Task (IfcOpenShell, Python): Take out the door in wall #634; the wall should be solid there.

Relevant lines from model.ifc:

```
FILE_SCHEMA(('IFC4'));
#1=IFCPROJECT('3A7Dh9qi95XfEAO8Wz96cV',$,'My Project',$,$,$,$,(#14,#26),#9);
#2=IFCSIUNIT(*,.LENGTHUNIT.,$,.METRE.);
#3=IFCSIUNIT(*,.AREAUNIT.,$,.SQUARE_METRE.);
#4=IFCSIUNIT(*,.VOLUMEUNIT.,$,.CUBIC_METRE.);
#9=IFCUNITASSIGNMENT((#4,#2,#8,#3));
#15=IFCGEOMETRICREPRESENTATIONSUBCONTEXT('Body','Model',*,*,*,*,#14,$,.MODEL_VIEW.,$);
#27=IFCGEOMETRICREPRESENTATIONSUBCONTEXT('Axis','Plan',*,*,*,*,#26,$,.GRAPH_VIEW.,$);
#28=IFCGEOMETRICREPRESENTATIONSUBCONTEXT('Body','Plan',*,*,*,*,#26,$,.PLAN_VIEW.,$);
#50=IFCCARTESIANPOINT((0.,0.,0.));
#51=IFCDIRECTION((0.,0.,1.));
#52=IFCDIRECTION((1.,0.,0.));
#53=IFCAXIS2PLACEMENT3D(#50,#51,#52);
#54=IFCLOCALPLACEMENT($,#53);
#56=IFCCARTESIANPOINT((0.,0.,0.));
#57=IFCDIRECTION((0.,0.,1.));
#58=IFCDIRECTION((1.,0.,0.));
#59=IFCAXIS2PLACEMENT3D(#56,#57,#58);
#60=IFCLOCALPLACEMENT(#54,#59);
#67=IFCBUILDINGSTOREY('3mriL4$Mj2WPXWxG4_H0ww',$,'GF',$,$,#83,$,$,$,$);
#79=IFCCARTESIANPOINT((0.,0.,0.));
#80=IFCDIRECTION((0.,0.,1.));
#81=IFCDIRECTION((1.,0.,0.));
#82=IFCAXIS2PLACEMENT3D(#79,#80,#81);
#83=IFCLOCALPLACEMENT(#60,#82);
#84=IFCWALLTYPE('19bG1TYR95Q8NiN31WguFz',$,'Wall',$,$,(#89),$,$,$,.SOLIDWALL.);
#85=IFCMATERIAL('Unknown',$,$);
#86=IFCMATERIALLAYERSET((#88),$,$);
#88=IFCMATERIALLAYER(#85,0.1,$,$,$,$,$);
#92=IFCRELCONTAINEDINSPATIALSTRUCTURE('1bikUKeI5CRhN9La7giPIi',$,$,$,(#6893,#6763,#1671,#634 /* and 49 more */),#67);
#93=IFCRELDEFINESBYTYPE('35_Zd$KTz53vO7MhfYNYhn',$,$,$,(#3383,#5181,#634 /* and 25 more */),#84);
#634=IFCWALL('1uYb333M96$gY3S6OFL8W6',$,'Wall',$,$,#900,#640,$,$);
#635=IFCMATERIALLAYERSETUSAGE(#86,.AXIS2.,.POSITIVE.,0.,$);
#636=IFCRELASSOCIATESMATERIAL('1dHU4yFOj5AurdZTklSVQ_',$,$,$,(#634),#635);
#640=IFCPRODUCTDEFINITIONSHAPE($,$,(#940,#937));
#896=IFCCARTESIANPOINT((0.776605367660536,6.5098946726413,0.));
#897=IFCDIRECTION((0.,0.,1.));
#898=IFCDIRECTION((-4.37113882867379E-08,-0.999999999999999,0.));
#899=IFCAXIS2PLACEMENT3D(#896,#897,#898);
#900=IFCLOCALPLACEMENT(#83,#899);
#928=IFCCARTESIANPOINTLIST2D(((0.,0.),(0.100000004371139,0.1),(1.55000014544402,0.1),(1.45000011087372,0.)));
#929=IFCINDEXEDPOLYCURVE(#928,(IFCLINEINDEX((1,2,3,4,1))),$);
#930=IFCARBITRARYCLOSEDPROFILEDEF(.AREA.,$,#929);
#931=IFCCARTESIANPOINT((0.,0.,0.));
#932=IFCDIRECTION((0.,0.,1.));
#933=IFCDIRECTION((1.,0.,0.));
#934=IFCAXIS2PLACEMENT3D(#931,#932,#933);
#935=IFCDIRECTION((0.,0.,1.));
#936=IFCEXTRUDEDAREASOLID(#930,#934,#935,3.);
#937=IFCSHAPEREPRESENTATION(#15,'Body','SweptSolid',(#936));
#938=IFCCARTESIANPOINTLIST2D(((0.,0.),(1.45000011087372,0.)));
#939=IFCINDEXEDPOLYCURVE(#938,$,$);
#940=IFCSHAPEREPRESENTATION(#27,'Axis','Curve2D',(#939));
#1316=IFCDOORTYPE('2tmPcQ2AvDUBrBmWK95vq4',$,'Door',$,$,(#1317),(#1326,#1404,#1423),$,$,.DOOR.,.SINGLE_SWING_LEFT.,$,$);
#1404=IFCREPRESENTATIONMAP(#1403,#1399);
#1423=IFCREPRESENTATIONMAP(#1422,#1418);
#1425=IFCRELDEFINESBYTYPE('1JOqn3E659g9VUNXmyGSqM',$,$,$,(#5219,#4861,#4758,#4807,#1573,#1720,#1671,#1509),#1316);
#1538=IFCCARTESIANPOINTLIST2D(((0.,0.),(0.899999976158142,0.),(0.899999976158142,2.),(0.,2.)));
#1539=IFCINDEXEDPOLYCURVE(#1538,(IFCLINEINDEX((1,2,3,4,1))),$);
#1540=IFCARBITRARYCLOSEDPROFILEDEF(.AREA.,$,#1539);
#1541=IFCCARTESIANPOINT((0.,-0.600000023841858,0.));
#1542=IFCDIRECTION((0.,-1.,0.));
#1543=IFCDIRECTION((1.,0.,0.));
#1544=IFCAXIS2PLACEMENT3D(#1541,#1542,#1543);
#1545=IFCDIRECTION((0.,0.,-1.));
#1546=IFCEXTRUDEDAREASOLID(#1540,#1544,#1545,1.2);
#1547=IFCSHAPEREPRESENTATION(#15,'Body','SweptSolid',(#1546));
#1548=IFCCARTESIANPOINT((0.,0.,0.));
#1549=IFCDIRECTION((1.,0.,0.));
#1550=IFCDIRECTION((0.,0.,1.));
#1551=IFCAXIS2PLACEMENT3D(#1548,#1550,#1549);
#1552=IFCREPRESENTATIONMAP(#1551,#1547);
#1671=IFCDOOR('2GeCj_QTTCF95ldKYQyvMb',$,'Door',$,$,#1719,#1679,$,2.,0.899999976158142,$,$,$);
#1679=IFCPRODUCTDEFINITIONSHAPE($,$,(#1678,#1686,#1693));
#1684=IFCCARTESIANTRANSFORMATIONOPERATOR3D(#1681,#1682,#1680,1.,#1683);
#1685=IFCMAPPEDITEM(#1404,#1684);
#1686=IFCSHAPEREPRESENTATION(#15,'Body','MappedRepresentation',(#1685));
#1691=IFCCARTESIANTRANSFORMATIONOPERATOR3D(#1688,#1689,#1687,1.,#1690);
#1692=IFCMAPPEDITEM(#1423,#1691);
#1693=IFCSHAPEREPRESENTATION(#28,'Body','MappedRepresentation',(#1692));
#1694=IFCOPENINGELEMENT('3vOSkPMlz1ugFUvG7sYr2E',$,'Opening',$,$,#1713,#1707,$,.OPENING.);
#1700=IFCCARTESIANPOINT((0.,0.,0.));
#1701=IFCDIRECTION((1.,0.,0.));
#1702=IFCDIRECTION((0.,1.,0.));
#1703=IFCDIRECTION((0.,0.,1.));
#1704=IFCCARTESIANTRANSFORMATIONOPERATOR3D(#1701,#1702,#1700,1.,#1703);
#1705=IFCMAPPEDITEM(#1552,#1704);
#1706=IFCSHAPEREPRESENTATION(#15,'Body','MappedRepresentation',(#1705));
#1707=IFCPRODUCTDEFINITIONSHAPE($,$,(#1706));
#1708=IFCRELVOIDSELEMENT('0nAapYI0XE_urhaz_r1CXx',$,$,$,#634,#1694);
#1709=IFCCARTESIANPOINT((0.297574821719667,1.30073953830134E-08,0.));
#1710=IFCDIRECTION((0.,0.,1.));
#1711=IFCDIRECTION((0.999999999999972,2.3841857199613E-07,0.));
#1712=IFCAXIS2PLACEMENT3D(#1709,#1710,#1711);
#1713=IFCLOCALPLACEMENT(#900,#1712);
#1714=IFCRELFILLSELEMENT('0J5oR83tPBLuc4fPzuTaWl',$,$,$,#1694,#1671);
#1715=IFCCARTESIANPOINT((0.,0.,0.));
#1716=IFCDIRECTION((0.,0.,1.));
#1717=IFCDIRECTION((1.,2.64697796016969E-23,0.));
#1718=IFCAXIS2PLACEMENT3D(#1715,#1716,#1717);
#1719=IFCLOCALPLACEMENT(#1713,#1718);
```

```python
import ifcopenshell
import ifcopenshell.api.feature
import ifcopenshell.api.root
import ifcopenshell.geom
import ifcopenshell.util.shape

model = ifcopenshell.open("model.ifc")
settings = ifcopenshell.geom.settings()


def volume(element):
    """Net volume in cubic metres, openings subtracted."""
    shape = ifcopenshell.geom.create_shape(settings, element)
    return ifcopenshell.util.shape.get_volume(shape.geometry)


door = model.by_guid("2GeCj_QTTCF95ldKYQyvMb")
opening = door.FillsVoids[0].RelatingOpeningElement
wall = opening.VoidsElements[0].RelatingBuildingElement
before = volume(wall)

ifcopenshell.api.root.remove_product(model, product=door)
ifcopenshell.api.feature.remove_feature(model, feature=opening)

after = volume(wall)

print(f"wall volume {before:.3f} -> {after:.3f} m3")

model.write("model_updated.ifc")
```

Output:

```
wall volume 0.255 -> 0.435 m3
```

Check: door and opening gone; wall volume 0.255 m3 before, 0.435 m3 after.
